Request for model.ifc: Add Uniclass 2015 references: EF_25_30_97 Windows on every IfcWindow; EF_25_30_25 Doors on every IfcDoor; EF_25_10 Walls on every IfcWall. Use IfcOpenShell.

First a look at what the model holds.

```python
import ifcopenshell

model = ifcopenshell.open("model.ifc")
print(model.schema)
print("classifications:", [c.Name for c in model.by_type("IfcClassification")])
for ifc_class in ("IfcDoor", "IfcRoof", "IfcStair", "IfcWall", "IfcWindow"):
    print(ifc_class, len(model.by_type(ifc_class)))
```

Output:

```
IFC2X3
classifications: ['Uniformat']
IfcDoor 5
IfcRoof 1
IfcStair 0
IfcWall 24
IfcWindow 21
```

```python
import ifcopenshell
import ifcopenshell.api.classification

model = ifcopenshell.open("model.ifc")

# IFC2X3 requires Source and Edition and has no link from the project to the system.
system = model.create_entity("IfcClassification", Source="NBS", Edition="2015", Name="Uniclass 2015")

codes = {
    "IfcWindow": ("EF_25_30_97", "Windows"),
    "IfcDoor": ("EF_25_30_25", "Doors"),
    "IfcWall": ("EF_25_10", "Walls"),
}
for ifc_class, (code, name) in codes.items():
    products = model.by_type(ifc_class)
    ifcopenshell.api.classification.add_reference(
        model, products=products, classification=system, identification=code, name=name
    )
    print(code, len(products))

model.write("model_updated.ifc")
```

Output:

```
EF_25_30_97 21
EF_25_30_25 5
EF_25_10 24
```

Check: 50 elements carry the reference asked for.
